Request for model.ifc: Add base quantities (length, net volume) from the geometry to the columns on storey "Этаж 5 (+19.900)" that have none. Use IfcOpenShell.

First a look at what the model holds.

```python
import ifcopenshell
import ifcopenshell.util.element
import ifcopenshell.util.unit

model = ifcopenshell.open("model.ifc")
print(model.schema)
for unit_type in ("LENGTHUNIT", "AREAUNIT", "VOLUMEUNIT"):
    print(unit_type, ifcopenshell.util.unit.calculate_unit_scale(model, unit_type))
storey = next(s for s in model.by_type("IfcBuildingStorey") if s.Name == "Этаж 5 (+19.900)")
columns = [e for e in ifcopenshell.util.element.get_decomposition(storey) if e.is_a("IfcColumn")]
for e in sorted(columns, key=lambda e: e.id()):
    print(e.id(), e.is_a(), e.Name, list(ifcopenshell.util.element.get_psets(e, qtos_only=True)), sep=" | ")
```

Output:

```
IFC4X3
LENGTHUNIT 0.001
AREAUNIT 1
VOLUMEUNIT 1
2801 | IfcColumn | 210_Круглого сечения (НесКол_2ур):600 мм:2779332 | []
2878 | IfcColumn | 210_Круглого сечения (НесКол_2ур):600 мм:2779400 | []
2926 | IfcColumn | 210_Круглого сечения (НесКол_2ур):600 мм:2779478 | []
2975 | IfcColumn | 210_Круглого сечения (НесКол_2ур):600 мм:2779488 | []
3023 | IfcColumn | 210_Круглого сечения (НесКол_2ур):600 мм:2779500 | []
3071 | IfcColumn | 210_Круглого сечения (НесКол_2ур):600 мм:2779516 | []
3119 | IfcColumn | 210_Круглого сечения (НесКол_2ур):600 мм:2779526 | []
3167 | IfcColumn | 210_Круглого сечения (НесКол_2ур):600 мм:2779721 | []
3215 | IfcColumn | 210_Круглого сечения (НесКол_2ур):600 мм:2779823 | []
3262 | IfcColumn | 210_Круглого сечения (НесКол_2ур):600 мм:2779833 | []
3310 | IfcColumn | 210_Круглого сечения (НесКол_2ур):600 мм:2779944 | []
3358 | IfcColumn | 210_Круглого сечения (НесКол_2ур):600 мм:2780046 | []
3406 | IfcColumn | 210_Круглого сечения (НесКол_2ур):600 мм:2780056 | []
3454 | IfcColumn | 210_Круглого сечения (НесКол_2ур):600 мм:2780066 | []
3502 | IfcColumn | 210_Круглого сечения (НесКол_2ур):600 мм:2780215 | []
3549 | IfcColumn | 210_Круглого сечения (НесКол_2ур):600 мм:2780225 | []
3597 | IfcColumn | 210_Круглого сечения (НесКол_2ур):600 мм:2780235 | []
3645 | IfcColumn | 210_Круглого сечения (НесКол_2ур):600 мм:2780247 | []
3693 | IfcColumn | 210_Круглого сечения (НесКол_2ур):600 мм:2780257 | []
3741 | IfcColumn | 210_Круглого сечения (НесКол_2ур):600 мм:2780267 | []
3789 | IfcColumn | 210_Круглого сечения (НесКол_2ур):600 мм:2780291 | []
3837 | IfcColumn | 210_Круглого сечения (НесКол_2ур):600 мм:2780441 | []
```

```python
import ifcopenshell
import ifcopenshell.api.pset
import ifcopenshell.geom
import ifcopenshell.util.element
import ifcopenshell.util.shape
import ifcopenshell.util.unit

model = ifcopenshell.open("model.ifc")
unit_scale = ifcopenshell.util.unit.calculate_unit_scale(model)
volume_scale = ifcopenshell.util.unit.calculate_unit_scale(model, "VOLUMEUNIT")
settings = ifcopenshell.geom.settings()

storey = next(s for s in model.by_type("IfcBuildingStorey") if s.Name == "Этаж 5 (+19.900)")
columns = [e for e in ifcopenshell.util.element.get_decomposition(storey) if e.is_a("IfcColumn")]

for e in sorted(columns, key=lambda e: e.id()):
    if ifcopenshell.util.element.get_psets(e, qtos_only=True, should_inherit=False):
        continue
    # Geometry comes back in metres, in the element's own axes.
    shape = ifcopenshell.geom.create_shape(settings, e)
    values = {
        "Length": ifcopenshell.util.shape.get_z(shape.geometry) / unit_scale,
        "NetVolume": ifcopenshell.util.shape.get_volume(shape.geometry) / volume_scale,
    }
    qto = ifcopenshell.api.pset.add_qto(model, product=e, name="Qto_ColumnBaseQuantities")
    ifcopenshell.api.pset.edit_qto(model, qto=qto, properties=values)
    print(e.id(), {k: round(v, 3) for k, v in values.items()})

model.write("model_updated.ifc")
```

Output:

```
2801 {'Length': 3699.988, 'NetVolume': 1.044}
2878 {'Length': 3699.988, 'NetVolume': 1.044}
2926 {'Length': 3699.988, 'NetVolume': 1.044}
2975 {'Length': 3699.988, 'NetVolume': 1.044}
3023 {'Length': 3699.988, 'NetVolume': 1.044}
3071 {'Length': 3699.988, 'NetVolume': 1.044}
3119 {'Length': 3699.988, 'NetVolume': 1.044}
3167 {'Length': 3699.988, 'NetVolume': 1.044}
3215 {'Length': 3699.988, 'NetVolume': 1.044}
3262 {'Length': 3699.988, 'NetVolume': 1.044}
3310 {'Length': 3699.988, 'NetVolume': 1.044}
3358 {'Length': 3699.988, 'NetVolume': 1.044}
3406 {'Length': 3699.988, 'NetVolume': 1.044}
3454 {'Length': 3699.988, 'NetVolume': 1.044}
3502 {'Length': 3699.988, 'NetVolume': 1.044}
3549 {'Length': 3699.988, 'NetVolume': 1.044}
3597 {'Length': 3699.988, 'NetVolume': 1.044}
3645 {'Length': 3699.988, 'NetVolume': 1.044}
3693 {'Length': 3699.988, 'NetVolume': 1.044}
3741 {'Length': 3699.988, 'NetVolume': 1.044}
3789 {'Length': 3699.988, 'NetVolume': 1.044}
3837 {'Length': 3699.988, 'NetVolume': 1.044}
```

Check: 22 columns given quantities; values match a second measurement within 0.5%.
